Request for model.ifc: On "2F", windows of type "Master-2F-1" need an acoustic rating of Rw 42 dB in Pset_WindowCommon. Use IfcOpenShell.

First a look at what the model holds.

```python
import ifcopenshell
import ifcopenshell.util.element

model = ifcopenshell.open("model.ifc")
print(model.schema)
storey = next(s for s in model.by_type("IfcBuildingStorey") if s.Name == "2F")
windows = [e for e in ifcopenshell.util.element.get_decomposition(storey) if e.is_a("IfcWindow")]
seen = {}
for e in windows:
    element_type = ifcopenshell.util.element.get_type(e)
    key = (element_type.Name if element_type != e and element_type else None, ifcopenshell.util.element.get_pset(e, "Pset_WindowCommon", "AcousticRating"))
    seen[key] = seen.get(key, 0) + 1
for (name, value), count in sorted(seen.items(), key=str):
    print(count, "x", name, "|", value)
```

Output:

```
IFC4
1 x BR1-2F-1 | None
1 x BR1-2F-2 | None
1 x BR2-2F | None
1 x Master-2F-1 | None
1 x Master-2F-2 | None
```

```python
import ifcopenshell
import ifcopenshell.api.pset
import ifcopenshell.util.element

model = ifcopenshell.open("model.ifc")

storey = next(s for s in model.by_type("IfcBuildingStorey") if s.Name == "2F")
windows = [e for e in ifcopenshell.util.element.get_decomposition(storey) if e.is_a("IfcWindow")]

count = 0
for e in windows:
    element_type = ifcopenshell.util.element.get_type(e)
    if element_type in (None, e) or element_type.Name != "Master-2F-1":
        continue
    # add_pset returns the element's existing set when there is one.
    pset = ifcopenshell.api.pset.add_pset(model, product=e, name="Pset_WindowCommon")
    ifcopenshell.api.pset.edit_pset(model, pset=pset, properties={"AcousticRating": "Rw 42 dB"})
    count += 1

print(count, "windows updated")

model.write("model_edited.ifc")
```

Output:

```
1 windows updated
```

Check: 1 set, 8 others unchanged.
